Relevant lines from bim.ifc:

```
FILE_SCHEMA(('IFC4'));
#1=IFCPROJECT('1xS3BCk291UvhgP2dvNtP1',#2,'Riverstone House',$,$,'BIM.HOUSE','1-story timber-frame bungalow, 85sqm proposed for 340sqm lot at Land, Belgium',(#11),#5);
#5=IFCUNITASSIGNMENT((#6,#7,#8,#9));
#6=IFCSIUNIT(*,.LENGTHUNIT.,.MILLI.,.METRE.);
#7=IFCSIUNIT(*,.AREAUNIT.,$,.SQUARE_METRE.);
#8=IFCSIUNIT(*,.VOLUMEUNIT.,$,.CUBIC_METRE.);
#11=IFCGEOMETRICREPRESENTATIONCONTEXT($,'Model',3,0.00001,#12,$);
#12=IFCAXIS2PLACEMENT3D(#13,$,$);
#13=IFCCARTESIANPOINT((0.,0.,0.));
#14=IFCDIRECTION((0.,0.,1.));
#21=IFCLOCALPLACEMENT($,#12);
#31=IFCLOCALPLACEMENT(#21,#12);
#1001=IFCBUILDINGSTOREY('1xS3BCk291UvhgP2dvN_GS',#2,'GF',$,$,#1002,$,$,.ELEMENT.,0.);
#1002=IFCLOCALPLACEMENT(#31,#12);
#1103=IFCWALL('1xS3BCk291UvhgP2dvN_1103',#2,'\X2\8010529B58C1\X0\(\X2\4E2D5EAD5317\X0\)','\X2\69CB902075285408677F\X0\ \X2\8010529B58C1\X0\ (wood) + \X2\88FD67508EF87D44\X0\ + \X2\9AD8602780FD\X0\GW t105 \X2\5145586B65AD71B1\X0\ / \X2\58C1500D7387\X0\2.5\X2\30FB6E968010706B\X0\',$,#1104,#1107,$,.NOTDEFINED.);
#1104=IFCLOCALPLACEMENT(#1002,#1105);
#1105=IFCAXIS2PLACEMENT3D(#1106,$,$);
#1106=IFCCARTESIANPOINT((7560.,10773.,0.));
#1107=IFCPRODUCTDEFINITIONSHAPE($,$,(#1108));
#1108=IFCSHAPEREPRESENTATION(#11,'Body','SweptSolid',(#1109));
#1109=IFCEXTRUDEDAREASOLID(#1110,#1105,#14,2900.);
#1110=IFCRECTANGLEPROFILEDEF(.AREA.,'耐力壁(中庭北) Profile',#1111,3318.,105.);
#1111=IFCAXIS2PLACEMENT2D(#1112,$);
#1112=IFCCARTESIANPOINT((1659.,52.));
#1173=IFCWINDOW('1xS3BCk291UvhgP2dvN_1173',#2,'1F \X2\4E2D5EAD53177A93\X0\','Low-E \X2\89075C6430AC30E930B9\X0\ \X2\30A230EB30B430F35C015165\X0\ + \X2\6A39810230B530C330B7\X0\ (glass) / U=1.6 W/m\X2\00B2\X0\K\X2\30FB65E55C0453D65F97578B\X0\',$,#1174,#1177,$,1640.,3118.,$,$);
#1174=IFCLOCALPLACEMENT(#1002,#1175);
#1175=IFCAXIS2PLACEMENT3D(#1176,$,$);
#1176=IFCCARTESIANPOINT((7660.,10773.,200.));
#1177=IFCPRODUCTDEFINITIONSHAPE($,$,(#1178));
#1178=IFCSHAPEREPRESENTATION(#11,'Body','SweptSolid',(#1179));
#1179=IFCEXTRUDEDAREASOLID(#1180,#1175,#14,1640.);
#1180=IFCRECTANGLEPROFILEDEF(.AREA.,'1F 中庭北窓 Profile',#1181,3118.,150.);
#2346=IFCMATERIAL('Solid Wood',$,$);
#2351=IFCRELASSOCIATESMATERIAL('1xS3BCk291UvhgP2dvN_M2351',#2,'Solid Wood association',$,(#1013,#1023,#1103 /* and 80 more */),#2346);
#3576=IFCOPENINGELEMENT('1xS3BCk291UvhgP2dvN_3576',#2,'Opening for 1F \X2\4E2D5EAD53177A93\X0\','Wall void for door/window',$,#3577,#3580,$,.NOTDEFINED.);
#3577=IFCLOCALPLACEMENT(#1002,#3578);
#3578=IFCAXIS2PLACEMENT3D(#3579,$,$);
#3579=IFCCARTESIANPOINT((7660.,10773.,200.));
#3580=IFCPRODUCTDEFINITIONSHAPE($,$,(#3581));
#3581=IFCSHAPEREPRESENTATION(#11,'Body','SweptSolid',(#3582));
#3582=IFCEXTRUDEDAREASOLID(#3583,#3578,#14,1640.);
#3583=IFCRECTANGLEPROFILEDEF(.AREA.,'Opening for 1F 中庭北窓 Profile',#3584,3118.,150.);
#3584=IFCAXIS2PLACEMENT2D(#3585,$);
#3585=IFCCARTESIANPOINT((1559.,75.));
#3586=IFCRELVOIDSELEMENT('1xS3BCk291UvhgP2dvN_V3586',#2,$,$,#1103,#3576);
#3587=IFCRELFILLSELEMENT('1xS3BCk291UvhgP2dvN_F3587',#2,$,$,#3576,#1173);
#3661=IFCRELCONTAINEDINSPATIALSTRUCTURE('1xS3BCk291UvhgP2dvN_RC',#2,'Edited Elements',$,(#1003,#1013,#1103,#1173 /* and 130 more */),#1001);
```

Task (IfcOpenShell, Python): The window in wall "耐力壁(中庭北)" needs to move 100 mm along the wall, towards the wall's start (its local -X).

```python
import ifcopenshell
import ifcopenshell.api.geometry
import ifcopenshell.util.placement
import ifcopenshell.util.unit

model = ifcopenshell.open("bim.ifc")
unit_scale = ifcopenshell.util.unit.calculate_unit_scale(model)

window = model.by_guid("1xS3BCk291UvhgP2dvN_1173")
opening = window.FillsVoids[0].RelatingOpeningElement
wall = opening.VoidsElements[0].RelatingBuildingElement

wall_matrix = ifcopenshell.util.placement.get_local_placement(wall.ObjectPlacement)
shift = wall_matrix[:3, 0] * -0.1 / unit_scale
before = ifcopenshell.util.placement.get_local_placement(window.ObjectPlacement)[:3, 3].copy()

# The window is not placed relative to its opening, so move both.
for product in (opening, window):
    matrix = ifcopenshell.util.placement.get_local_placement(product.ObjectPlacement)
    matrix[:3, 3] += shift
    ifcopenshell.api.geometry.edit_object_placement(model, product=product, matrix=matrix, is_si=False)

after = ifcopenshell.util.placement.get_local_placement(window.ObjectPlacement)[:3, 3]
print("window moved by", (after - before).round(3) + 0.0)

model.write("bim_v2.ifc")
```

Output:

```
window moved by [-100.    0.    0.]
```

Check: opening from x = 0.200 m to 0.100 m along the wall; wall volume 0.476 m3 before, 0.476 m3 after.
